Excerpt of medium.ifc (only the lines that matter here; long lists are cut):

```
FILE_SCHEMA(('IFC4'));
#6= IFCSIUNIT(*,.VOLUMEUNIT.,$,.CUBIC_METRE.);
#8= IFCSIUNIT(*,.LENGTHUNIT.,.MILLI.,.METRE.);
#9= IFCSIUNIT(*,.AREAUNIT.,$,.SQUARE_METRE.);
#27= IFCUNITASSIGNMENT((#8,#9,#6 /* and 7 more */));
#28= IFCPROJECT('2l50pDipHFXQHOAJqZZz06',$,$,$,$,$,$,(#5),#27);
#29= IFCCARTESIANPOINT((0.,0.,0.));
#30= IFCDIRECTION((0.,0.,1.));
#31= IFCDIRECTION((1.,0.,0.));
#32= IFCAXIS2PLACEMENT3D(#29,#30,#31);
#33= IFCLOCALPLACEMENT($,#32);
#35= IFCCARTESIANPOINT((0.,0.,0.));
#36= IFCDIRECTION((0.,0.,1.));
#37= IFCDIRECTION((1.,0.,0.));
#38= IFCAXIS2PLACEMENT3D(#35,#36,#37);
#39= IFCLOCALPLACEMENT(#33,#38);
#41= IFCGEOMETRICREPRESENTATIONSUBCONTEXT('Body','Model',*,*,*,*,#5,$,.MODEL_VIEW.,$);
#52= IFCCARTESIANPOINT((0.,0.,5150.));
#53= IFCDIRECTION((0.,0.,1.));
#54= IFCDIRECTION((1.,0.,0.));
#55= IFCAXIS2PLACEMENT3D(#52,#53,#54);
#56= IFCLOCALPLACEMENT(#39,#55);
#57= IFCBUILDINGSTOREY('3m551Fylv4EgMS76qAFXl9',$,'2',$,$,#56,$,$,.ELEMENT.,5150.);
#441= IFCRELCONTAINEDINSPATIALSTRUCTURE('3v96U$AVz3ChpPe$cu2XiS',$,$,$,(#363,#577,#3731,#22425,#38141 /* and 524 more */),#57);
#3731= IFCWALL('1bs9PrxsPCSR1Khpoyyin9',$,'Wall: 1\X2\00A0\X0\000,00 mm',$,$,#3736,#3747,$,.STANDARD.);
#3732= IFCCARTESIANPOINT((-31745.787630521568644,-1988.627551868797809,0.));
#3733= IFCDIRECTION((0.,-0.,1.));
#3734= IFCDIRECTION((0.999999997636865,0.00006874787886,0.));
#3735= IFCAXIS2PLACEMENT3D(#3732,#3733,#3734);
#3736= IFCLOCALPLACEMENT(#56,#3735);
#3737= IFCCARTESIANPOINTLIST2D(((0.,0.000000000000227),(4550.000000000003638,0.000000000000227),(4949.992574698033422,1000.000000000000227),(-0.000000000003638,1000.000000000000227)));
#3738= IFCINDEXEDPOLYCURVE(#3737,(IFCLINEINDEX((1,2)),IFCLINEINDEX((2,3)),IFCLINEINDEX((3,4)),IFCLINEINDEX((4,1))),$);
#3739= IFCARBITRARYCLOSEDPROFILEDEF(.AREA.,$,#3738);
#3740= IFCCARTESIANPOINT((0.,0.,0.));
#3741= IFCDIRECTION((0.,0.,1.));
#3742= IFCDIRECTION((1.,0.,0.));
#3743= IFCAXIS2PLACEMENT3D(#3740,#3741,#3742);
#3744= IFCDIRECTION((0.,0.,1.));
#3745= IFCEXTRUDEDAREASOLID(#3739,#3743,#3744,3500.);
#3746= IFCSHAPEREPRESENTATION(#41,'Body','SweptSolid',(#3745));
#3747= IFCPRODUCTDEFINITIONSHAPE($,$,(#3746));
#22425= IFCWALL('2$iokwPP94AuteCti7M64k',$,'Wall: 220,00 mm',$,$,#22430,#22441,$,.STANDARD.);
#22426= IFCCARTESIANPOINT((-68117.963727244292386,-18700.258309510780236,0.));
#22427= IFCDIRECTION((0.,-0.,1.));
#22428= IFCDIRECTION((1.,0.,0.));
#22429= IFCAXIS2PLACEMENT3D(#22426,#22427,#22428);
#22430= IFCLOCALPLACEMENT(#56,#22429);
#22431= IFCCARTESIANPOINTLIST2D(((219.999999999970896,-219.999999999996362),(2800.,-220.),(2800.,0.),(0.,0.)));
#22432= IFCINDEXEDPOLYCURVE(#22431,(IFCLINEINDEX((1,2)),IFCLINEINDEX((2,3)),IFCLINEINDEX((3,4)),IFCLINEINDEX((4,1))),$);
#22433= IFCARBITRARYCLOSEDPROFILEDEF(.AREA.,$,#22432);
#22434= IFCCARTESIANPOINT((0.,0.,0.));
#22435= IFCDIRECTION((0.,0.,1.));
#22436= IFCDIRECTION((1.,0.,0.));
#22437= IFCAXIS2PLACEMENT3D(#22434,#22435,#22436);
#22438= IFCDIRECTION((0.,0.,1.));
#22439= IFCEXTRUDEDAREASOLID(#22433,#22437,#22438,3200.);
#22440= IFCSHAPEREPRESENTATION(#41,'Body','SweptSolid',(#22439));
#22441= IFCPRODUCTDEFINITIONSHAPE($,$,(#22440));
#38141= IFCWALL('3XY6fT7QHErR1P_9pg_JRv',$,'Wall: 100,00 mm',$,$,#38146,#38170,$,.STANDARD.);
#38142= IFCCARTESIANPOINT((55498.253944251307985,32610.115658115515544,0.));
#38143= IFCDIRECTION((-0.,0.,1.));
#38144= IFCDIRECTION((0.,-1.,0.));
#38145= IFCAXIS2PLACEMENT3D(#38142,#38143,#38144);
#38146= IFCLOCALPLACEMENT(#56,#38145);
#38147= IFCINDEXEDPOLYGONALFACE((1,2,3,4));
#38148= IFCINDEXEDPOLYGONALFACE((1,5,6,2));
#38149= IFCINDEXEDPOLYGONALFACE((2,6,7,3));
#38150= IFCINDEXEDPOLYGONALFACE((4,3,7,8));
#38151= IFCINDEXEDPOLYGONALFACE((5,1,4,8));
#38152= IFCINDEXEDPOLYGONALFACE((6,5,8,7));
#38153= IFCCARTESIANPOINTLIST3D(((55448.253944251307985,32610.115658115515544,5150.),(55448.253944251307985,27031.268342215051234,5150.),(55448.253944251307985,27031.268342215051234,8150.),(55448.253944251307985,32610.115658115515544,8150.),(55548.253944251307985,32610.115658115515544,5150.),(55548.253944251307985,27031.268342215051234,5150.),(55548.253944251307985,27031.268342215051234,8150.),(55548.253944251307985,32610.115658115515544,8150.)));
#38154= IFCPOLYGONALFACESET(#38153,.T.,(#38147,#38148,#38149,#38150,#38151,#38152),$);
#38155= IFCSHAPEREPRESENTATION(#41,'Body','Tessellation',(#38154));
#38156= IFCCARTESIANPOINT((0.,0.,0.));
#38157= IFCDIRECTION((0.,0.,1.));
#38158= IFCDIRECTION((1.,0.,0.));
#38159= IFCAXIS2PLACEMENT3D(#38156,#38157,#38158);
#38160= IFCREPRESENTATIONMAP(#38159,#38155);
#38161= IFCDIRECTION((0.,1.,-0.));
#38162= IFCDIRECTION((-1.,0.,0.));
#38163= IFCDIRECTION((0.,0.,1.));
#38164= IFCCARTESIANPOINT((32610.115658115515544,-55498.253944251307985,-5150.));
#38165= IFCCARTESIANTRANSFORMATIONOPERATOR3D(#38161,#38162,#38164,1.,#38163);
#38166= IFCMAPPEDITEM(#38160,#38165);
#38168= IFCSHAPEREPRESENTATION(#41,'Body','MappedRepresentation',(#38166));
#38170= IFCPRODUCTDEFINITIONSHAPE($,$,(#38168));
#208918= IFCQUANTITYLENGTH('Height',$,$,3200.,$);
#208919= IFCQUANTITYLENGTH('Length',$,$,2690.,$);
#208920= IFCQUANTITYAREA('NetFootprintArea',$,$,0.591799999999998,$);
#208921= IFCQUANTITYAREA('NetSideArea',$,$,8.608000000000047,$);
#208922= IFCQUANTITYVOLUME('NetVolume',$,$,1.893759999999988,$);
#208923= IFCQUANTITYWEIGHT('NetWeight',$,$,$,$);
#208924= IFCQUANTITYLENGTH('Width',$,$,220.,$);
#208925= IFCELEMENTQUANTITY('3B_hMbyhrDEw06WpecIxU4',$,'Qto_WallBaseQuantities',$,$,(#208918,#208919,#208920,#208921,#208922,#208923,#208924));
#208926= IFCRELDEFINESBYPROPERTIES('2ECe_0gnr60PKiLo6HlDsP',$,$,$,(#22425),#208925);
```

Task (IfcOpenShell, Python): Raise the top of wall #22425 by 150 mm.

```python
import ifcopenshell
import ifcopenshell.api.pset
import ifcopenshell.geom
import ifcopenshell.util.element
import ifcopenshell.util.representation
import ifcopenshell.util.shape
import ifcopenshell.util.unit

model = ifcopenshell.open("medium.ifc")
area_scale = ifcopenshell.util.unit.calculate_unit_scale(model, "AREAUNIT")
volume_scale = ifcopenshell.util.unit.calculate_unit_scale(model, "VOLUMEUNIT")
settings = ifcopenshell.geom.settings()


def volume(element):
    """Net volume in cubic metres, openings subtracted."""
    shape = ifcopenshell.geom.create_shape(settings, element)
    return ifcopenshell.util.shape.get_volume(shape.geometry)


wall = model.by_guid("2$iokwPP94AuteCti7M64k")
before = volume(wall)

body = ifcopenshell.util.representation.get_representation(wall, "Model", "Body")
solid = body.Items[0]
old_height = solid.Depth
solid.Depth += 150.0
after = volume(wall)
thickness = 0.22  # wall thickness in metres

# Update the stored height, areas and volumes.
qto = model.by_id(ifcopenshell.util.element.get_pset(wall, "Qto_WallBaseQuantities", should_inherit=False)["id"])
ifcopenshell.api.pset.edit_qto(model, qto=qto, properties={
    "Height": solid.Depth,
    "NetSideArea": after / thickness / area_scale,
    "NetVolume": after / volume_scale,
})

print(f"height {old_height:g} -> {solid.Depth:g}, volume {before:.3f} -> {after:.3f} m3")

model.write("medium_rev.ifc")
```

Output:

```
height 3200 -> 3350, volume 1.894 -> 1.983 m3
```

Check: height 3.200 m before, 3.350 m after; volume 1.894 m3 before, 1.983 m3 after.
